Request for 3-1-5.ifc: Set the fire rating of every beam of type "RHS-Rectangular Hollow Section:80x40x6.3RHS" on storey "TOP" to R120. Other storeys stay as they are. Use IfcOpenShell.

First a look at what the model holds.

```python
import ifcopenshell
import ifcopenshell.util.element

model = ifcopenshell.open("3-1-5.ifc")
print(model.schema)
storey = next(s for s in model.by_type("IfcBuildingStorey") if s.Name == "TOP")
beams = [e for e in ifcopenshell.util.element.get_decomposition(storey) if e.is_a("IfcBeam")]
seen = {}
for e in beams:
    element_type = ifcopenshell.util.element.get_type(e)
    key = (element_type.Name if element_type != e and element_type else None, ifcopenshell.util.element.get_pset(e, "Pset_BeamCommon", "FireRating"))
    seen[key] = seen.get(key, 0) + 1
for (name, value), count in sorted(seen.items(), key=str):
    print(count, "x", name, "|", value)
```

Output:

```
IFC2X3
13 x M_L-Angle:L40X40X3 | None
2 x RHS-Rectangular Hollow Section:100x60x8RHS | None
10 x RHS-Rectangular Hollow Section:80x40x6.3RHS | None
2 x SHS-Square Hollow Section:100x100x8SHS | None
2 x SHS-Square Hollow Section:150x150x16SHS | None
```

```python
import ifcopenshell
import ifcopenshell.api.pset
import ifcopenshell.util.element

model = ifcopenshell.open("3-1-5.ifc")

storey = next(s for s in model.by_type("IfcBuildingStorey") if s.Name == "TOP")
beams = [e for e in ifcopenshell.util.element.get_decomposition(storey) if e.is_a("IfcBeam")]

count = 0
for e in beams:
    element_type = ifcopenshell.util.element.get_type(e)
    if element_type in (None, e) or element_type.Name != "RHS-Rectangular Hollow Section:80x40x6.3RHS":
        continue
    # add_pset returns the element's existing set when there is one.
    pset = ifcopenshell.api.pset.add_pset(model, product=e, name="Pset_BeamCommon")
    ifcopenshell.api.pset.edit_pset(model, pset=pset, properties={"FireRating": "R120"})
    count += 1

print(count, "beams updated")

model.write("3-1-5_edited.ifc")
```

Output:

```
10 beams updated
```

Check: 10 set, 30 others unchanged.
